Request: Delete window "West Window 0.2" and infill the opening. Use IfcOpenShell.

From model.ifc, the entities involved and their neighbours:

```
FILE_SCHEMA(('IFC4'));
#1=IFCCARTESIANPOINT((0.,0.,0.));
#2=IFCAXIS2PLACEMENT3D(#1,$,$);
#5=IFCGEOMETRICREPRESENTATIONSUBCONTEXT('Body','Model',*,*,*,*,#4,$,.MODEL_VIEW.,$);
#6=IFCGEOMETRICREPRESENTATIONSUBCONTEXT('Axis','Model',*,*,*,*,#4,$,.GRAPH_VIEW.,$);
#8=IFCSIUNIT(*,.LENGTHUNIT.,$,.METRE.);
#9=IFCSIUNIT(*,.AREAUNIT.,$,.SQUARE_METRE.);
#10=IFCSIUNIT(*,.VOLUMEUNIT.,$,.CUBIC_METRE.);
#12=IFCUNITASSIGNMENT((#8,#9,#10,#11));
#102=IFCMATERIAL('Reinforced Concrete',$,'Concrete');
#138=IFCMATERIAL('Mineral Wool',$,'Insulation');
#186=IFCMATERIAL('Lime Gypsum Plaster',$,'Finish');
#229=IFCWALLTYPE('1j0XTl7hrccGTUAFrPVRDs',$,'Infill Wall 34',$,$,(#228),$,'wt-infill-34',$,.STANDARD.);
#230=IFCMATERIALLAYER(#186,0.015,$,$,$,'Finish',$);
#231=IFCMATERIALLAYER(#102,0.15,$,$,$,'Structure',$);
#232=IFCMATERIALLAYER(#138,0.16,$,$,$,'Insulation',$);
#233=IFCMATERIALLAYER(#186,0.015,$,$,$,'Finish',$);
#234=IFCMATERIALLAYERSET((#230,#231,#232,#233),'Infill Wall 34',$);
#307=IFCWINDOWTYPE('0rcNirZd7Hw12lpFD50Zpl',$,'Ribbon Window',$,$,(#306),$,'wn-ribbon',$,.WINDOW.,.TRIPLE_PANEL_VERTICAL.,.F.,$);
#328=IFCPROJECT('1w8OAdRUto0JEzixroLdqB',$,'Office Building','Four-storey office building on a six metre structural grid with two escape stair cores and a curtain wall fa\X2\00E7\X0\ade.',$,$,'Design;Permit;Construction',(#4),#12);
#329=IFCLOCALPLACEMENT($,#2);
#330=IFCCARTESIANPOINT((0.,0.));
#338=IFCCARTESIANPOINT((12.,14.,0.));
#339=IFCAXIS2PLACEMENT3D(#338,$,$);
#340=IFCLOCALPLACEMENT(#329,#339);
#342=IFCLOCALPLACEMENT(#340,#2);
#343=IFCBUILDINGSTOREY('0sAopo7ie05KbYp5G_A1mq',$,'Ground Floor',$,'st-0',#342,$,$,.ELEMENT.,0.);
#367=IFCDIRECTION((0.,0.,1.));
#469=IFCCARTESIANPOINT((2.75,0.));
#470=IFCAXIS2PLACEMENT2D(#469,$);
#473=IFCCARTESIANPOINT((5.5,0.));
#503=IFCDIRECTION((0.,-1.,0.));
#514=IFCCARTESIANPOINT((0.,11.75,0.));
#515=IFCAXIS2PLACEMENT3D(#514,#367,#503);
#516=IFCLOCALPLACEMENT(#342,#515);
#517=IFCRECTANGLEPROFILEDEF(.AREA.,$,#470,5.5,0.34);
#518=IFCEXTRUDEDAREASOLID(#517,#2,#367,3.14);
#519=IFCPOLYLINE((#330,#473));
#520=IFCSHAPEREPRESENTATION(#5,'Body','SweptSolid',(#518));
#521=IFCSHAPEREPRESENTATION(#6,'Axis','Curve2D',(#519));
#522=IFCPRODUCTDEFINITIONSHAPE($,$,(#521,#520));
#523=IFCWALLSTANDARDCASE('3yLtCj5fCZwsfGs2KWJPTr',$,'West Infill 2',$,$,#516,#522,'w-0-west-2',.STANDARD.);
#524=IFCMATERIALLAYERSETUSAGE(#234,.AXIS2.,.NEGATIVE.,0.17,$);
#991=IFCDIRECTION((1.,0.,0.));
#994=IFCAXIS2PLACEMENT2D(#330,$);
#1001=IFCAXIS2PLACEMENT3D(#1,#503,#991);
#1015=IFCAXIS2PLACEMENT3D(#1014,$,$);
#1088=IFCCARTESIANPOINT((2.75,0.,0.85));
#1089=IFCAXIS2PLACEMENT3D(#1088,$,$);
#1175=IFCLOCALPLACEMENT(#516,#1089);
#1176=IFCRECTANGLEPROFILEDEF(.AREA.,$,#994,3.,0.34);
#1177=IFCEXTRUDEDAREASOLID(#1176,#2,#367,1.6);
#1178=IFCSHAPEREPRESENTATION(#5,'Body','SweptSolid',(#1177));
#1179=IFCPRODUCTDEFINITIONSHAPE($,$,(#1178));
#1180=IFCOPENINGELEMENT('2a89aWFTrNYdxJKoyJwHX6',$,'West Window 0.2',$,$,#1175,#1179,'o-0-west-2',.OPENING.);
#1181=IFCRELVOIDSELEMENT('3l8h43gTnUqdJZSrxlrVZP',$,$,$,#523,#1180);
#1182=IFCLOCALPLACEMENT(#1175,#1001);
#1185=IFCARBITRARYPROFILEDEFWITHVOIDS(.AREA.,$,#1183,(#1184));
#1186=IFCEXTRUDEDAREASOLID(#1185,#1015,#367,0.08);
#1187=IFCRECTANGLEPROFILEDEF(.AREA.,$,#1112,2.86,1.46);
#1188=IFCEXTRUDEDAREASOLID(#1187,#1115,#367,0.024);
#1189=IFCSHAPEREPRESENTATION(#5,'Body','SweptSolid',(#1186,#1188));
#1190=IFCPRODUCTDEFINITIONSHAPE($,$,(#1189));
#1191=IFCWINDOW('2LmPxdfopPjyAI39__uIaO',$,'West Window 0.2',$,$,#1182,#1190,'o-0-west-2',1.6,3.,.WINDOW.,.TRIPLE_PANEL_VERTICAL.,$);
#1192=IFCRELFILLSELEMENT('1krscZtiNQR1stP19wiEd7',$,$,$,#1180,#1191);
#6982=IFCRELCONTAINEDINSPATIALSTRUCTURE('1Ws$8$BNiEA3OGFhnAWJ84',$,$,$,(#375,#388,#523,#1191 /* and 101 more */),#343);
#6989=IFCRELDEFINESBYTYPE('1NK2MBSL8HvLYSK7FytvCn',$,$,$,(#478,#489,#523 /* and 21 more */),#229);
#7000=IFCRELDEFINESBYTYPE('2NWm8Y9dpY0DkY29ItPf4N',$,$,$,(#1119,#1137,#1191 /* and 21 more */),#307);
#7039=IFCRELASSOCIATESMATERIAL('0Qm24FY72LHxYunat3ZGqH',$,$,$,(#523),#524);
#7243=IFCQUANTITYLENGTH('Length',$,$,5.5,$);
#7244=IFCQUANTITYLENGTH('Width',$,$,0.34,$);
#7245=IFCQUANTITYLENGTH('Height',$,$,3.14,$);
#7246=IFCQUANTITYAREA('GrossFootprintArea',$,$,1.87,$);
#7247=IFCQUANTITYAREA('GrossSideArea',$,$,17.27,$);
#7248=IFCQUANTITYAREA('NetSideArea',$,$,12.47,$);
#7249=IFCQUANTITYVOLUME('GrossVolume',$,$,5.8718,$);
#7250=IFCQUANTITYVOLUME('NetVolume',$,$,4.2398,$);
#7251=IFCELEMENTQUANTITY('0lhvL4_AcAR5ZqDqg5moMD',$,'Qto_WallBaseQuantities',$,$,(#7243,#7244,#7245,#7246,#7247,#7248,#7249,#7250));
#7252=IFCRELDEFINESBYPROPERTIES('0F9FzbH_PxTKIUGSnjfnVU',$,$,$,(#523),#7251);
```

```python
import ifcopenshell
import ifcopenshell.api.feature
import ifcopenshell.api.pset
import ifcopenshell.api.root
import ifcopenshell.geom
import ifcopenshell.util.element
import ifcopenshell.util.shape
import ifcopenshell.util.unit

model = ifcopenshell.open("model.ifc")
area_scale = ifcopenshell.util.unit.calculate_unit_scale(model, "AREAUNIT")
volume_scale = ifcopenshell.util.unit.calculate_unit_scale(model, "VOLUMEUNIT")
settings = ifcopenshell.geom.settings()


def volume(element):
    """Net volume in cubic metres, openings subtracted."""
    shape = ifcopenshell.geom.create_shape(settings, element)
    return ifcopenshell.util.shape.get_volume(shape.geometry)


window = model.by_guid("2LmPxdfopPjyAI39__uIaO")
opening = window.FillsVoids[0].RelatingOpeningElement
wall = opening.VoidsElements[0].RelatingBuildingElement
before = volume(wall)

ifcopenshell.api.root.remove_product(model, product=window)
ifcopenshell.api.feature.remove_feature(model, feature=opening)

after = volume(wall)
thickness = 0.34  # wall thickness in metres

# Update the wall's stored quantities.
qto = model.by_id(ifcopenshell.util.element.get_pset(wall, "Qto_WallBaseQuantities", should_inherit=False)["id"])
ifcopenshell.api.pset.edit_qto(model, qto=qto, properties={
    "NetSideArea": after / thickness / area_scale,
    "NetVolume": after / volume_scale,
})

print(f"wall volume {before:.3f} -> {after:.3f} m3")

model.write("model_rev.ifc")
```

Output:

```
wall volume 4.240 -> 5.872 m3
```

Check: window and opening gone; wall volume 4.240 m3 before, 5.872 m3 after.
